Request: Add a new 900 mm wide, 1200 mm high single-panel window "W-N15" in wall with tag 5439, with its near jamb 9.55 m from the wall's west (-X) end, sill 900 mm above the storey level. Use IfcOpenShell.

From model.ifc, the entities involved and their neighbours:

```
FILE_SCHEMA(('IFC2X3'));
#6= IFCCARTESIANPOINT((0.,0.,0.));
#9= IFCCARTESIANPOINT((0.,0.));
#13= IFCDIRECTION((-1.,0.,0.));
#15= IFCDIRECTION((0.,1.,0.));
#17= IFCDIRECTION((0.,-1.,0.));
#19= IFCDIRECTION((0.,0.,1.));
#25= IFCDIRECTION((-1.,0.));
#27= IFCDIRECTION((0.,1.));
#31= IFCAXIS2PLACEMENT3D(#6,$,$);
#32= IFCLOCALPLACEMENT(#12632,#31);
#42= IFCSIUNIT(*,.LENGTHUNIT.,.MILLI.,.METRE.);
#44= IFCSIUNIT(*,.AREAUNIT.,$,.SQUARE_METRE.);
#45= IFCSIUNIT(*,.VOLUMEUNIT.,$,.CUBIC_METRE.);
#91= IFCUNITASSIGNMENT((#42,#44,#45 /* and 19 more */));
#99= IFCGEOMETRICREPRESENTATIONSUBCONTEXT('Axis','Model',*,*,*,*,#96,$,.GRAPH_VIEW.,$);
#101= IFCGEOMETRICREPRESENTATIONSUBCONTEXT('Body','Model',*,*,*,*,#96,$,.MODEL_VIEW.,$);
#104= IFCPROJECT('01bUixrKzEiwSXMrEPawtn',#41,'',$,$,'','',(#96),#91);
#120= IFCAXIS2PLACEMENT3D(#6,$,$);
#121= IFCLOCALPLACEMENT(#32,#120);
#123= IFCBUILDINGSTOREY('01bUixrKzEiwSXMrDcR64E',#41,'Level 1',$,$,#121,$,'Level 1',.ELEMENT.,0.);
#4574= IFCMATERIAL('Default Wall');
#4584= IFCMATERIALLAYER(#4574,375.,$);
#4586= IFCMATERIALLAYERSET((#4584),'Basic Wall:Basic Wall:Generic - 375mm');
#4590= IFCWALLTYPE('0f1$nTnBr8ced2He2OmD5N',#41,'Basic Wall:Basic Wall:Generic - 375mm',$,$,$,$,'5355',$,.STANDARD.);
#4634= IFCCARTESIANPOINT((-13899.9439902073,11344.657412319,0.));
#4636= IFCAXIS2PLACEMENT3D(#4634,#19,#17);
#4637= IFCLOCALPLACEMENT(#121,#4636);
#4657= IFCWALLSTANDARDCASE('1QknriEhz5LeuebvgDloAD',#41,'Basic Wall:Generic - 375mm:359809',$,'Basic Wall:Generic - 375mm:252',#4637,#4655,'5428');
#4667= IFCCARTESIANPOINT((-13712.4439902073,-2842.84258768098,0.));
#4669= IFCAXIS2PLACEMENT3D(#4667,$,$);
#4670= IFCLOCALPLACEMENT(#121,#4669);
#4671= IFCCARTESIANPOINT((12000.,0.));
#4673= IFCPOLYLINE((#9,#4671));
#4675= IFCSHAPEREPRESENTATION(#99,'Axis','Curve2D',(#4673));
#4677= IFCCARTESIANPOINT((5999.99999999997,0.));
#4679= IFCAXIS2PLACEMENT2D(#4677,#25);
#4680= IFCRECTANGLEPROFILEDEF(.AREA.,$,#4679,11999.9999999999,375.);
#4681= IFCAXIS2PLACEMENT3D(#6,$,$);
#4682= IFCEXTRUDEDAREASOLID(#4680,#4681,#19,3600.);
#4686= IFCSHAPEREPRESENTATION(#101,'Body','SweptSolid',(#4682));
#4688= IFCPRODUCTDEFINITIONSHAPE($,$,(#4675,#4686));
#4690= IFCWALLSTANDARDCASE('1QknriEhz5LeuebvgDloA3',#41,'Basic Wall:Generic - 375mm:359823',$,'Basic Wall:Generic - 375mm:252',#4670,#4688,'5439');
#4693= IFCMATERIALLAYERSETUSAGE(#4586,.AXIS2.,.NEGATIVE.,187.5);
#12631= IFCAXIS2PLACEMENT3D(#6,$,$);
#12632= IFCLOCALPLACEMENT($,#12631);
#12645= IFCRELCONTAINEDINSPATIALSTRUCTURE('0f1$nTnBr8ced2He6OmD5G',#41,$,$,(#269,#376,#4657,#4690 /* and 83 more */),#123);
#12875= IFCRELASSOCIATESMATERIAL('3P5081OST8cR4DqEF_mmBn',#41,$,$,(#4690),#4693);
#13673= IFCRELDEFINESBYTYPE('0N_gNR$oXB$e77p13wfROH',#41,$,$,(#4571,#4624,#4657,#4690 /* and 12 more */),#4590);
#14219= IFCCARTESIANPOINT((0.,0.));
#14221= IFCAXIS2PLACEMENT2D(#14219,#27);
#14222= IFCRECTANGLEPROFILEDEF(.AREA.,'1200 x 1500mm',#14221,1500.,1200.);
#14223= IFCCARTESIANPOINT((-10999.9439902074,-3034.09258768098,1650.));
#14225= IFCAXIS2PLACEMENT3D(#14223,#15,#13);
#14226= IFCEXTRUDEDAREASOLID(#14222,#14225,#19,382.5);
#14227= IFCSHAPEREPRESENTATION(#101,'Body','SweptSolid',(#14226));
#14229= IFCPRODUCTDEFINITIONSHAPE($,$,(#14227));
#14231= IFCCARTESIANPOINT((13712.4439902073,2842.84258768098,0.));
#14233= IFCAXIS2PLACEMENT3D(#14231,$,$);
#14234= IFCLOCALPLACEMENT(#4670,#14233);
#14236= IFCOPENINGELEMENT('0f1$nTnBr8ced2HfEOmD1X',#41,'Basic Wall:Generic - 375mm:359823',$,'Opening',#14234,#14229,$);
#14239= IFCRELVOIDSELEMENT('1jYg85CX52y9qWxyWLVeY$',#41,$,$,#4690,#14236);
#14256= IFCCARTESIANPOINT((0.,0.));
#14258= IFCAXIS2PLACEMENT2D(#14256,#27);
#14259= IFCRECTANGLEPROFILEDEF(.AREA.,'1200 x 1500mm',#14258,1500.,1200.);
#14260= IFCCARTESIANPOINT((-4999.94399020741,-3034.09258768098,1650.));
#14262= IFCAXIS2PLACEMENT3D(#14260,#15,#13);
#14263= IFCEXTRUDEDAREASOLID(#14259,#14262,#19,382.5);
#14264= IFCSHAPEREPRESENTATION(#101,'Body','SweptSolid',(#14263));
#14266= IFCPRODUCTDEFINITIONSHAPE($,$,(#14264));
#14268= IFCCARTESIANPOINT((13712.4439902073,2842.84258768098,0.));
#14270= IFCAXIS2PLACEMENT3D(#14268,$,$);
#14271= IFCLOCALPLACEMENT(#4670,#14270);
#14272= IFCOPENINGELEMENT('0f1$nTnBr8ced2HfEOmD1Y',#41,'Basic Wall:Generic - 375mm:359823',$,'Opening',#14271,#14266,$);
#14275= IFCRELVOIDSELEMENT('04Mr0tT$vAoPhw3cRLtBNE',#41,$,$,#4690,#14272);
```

```python
import numpy as np
import ifcopenshell
import ifcopenshell.api.feature
import ifcopenshell.api.geometry
import ifcopenshell.api.root
import ifcopenshell.api.spatial
import ifcopenshell.api.type
import ifcopenshell.geom
import ifcopenshell.util.element
import ifcopenshell.util.placement
import ifcopenshell.util.representation
import ifcopenshell.util.shape
import ifcopenshell.util.unit

model = ifcopenshell.open("model.ifc")
unit_scale = ifcopenshell.util.unit.calculate_unit_scale(model)
settings = ifcopenshell.geom.settings()


def volume(element):
    """Net volume in cubic metres, openings subtracted."""
    shape = ifcopenshell.geom.create_shape(settings, element)
    return ifcopenshell.util.shape.get_volume(shape.geometry)


wall = model.by_guid("1QknriEhz5LeuebvgDloA3")
storey = ifcopenshell.util.element.get_container(wall, ifc_class="IfcBuildingStorey")
context = ifcopenshell.util.representation.get_context(model, "Model", "Body", "MODEL_VIEW")
before = volume(wall)

width, height, from_end, sill = 0.9, 1.2, 9.55, 0.9  # metres

# The wall runs along its own X axis, and the end named is its -X end.
wall_shape = ifcopenshell.geom.create_shape(settings, wall)
x, y, z = ifcopenshell.util.shape.get_vertices(wall_shape.geometry).T
start = x.min() + from_end
face, thickness = float(y.min()), float(y.max() - y.min())
wall_matrix = ifcopenshell.util.placement.get_local_placement(wall.ObjectPlacement)
level = ifcopenshell.util.placement.get_local_placement(storey.ObjectPlacement)[2, 3]


def in_wall(x, y):
    """Placement at x, y metres in the wall's axes, at sill height."""
    matrix = wall_matrix.copy()
    matrix[:, 3] = wall_matrix @ np.array([x / unit_scale, y / unit_scale, 0.0, 1.0])
    matrix[2, 3] = level + sill / unit_scale
    return matrix


# Opening: a box that overshoots both wall faces by 50 mm.
opening = ifcopenshell.api.root.create_entity(model, ifc_class="IfcOpeningElement")
box = ifcopenshell.api.geometry.add_wall_representation(
    model, context=context, length=width, height=height, thickness=thickness + 0.1
)
ifcopenshell.api.geometry.assign_representation(model, product=opening, representation=box)
ifcopenshell.api.geometry.edit_object_placement(model, product=opening, matrix=in_wall(start, face - 0.05), is_si=False)
ifcopenshell.api.feature.add_feature(model, feature=opening, element=wall)

window = ifcopenshell.api.root.create_entity(model, ifc_class="IfcWindow", name="W-N15")
window.OverallWidth, window.OverallHeight = width / unit_scale, height / unit_scale
body = ifcopenshell.api.geometry.add_window_representation(
    model,
    context=context,
    overall_width=window.OverallWidth,
    overall_height=window.OverallHeight,
    partition_type="SINGLE_PANEL",
)
ifcopenshell.api.geometry.assign_representation(model, product=window, representation=body)
ifcopenshell.api.spatial.assign_container(model, products=[window], relating_structure=storey)
fills = ifcopenshell.api.feature.add_filling(model, opening=opening, element=window)
fills.OwnerHistory = window.OwnerHistory  # required in IFC2X3

# IFC2X3 keeps the operation on the window style.
style = ifcopenshell.api.root.create_entity(model, ifc_class="IfcWindowStyle", name="W-N15")
style.OperationType, style.ConstructionType = "SINGLE_PANEL", "NOTDEFINED"
style.ParameterTakesPrecedence = style.Sizeable = False
ifcopenshell.api.type.assign_type(model, related_objects=[window], relating_type=style)

# Centre the window in the wall's thickness.
ifcopenshell.api.geometry.edit_object_placement(model, product=window, matrix=in_wall(start, face), is_si=False)
window_shape = ifcopenshell.geom.create_shape(settings, window)
depth = ifcopenshell.util.shape.get_vertices(window_shape.geometry)[:, 1]
offset = face + thickness / 2 - (depth.min() + depth.max()) / 2
ifcopenshell.api.geometry.edit_object_placement(model, product=window, matrix=in_wall(start, offset), is_si=False)

after = volume(wall)

print(f"wall volume {before:.3f} -> {after:.3f} m3")

model.write("model-out.ifc")
```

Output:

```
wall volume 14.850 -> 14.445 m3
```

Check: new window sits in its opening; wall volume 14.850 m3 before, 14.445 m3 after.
